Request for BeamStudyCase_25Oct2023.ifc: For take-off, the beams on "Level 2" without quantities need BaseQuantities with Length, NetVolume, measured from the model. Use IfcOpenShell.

First a look at what the model holds.

```python
import ifcopenshell
import ifcopenshell.util.element
import ifcopenshell.util.unit

model = ifcopenshell.open("BeamStudyCase_25Oct2023.ifc")
print(model.schema)
for unit_type in ("LENGTHUNIT", "AREAUNIT", "VOLUMEUNIT"):
    print(unit_type, ifcopenshell.util.unit.calculate_unit_scale(model, unit_type))
storey = next(s for s in model.by_type("IfcBuildingStorey") if s.Name == "Level 2")
beams = [e for e in ifcopenshell.util.element.get_decomposition(storey) if e.is_a("IfcBeam")]
for e in sorted(beams, key=lambda e: e.id()):
    print(e.id(), e.is_a(), e.Name, list(ifcopenshell.util.element.get_psets(e, qtos_only=True)), sep=" | ")
```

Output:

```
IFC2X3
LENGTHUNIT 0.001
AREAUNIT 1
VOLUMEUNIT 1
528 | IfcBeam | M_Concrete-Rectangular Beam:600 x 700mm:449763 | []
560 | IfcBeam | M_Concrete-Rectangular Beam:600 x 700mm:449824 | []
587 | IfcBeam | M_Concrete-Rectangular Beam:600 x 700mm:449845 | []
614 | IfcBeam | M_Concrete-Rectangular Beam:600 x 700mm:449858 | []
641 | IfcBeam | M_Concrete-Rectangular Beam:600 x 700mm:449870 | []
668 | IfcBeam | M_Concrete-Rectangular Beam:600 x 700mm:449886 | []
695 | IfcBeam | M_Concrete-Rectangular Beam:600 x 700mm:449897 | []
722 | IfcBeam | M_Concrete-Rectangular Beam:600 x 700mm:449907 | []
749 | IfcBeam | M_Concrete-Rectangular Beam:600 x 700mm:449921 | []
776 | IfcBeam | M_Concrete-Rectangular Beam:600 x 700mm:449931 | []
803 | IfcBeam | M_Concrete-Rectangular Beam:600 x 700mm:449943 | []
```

```python
import ifcopenshell
import ifcopenshell.api.pset
import ifcopenshell.geom
import ifcopenshell.util.element
import ifcopenshell.util.shape
import ifcopenshell.util.unit

model = ifcopenshell.open("BeamStudyCase_25Oct2023.ifc")
unit_scale = ifcopenshell.util.unit.calculate_unit_scale(model)
volume_scale = ifcopenshell.util.unit.calculate_unit_scale(model, "VOLUMEUNIT")
settings = ifcopenshell.geom.settings()

storey = next(s for s in model.by_type("IfcBuildingStorey") if s.Name == "Level 2")
beams = [e for e in ifcopenshell.util.element.get_decomposition(storey) if e.is_a("IfcBeam")]

for e in sorted(beams, key=lambda e: e.id()):
    if ifcopenshell.util.element.get_psets(e, qtos_only=True, should_inherit=False):
        continue
    # Geometry comes back in metres, in the element's own axes.
    shape = ifcopenshell.geom.create_shape(settings, e)
    values = {
        "Length": ifcopenshell.util.shape.get_max_xyz(shape.geometry) / unit_scale,
        "NetVolume": ifcopenshell.util.shape.get_volume(shape.geometry) / volume_scale,
    }
    qto = ifcopenshell.api.pset.add_qto(model, product=e, name="BaseQuantities")
    ifcopenshell.api.pset.edit_qto(model, qto=qto, properties=values)
    print(e.id(), {k: round(v, 3) for k, v in values.items()})

model.write("BeamStudyCase_25Oct2023_v2.ifc")
```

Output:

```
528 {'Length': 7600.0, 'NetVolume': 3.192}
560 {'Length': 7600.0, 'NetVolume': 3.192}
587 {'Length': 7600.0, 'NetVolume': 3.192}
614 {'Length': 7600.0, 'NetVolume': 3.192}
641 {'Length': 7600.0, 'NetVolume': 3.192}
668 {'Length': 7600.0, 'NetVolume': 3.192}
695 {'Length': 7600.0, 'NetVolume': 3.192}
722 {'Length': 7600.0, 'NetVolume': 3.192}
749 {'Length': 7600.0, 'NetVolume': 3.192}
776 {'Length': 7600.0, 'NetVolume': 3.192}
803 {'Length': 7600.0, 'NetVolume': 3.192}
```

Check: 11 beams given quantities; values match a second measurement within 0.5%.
